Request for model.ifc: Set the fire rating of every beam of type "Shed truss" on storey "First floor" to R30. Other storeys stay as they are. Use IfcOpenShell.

First a look at what the model holds.

```python
import ifcopenshell
import ifcopenshell.util.element

model = ifcopenshell.open("model.ifc")
print(model.schema)
storey = next(s for s in model.by_type("IfcBuildingStorey") if s.Name == "First floor")
beams = [e for e in ifcopenshell.util.element.get_decomposition(storey) if e.is_a("IfcBeam")]
seen = {}
for e in beams:
    element_type = ifcopenshell.util.element.get_type(e)
    key = (element_type.Name if element_type != e and element_type else None, ifcopenshell.util.element.get_pset(e, "Pset_BeamCommon", "FireRating"))
    seen[key] = seen.get(key, 0) + 1
for (name, value), count in sorted(seen.items(), key=str):
    print(count, "x", name, "|", value)
```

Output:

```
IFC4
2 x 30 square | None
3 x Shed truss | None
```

```python
import ifcopenshell
import ifcopenshell.api.pset
import ifcopenshell.util.element

model = ifcopenshell.open("model.ifc")

storey = next(s for s in model.by_type("IfcBuildingStorey") if s.Name == "First floor")
beams = [e for e in ifcopenshell.util.element.get_decomposition(storey) if e.is_a("IfcBeam")]

count = 0
for e in beams:
    element_type = ifcopenshell.util.element.get_type(e)
    if element_type in (None, e) or element_type.Name != "Shed truss":
        continue
    # add_pset returns the element's existing set when there is one.
    pset = ifcopenshell.api.pset.add_pset(model, product=e, name="Pset_BeamCommon")
    ifcopenshell.api.pset.edit_pset(model, pset=pset, properties={"FireRating": "R30"})
    count += 1

print(count, "beams updated")

model.write("model_edited.ifc")
```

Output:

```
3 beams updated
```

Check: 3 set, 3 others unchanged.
